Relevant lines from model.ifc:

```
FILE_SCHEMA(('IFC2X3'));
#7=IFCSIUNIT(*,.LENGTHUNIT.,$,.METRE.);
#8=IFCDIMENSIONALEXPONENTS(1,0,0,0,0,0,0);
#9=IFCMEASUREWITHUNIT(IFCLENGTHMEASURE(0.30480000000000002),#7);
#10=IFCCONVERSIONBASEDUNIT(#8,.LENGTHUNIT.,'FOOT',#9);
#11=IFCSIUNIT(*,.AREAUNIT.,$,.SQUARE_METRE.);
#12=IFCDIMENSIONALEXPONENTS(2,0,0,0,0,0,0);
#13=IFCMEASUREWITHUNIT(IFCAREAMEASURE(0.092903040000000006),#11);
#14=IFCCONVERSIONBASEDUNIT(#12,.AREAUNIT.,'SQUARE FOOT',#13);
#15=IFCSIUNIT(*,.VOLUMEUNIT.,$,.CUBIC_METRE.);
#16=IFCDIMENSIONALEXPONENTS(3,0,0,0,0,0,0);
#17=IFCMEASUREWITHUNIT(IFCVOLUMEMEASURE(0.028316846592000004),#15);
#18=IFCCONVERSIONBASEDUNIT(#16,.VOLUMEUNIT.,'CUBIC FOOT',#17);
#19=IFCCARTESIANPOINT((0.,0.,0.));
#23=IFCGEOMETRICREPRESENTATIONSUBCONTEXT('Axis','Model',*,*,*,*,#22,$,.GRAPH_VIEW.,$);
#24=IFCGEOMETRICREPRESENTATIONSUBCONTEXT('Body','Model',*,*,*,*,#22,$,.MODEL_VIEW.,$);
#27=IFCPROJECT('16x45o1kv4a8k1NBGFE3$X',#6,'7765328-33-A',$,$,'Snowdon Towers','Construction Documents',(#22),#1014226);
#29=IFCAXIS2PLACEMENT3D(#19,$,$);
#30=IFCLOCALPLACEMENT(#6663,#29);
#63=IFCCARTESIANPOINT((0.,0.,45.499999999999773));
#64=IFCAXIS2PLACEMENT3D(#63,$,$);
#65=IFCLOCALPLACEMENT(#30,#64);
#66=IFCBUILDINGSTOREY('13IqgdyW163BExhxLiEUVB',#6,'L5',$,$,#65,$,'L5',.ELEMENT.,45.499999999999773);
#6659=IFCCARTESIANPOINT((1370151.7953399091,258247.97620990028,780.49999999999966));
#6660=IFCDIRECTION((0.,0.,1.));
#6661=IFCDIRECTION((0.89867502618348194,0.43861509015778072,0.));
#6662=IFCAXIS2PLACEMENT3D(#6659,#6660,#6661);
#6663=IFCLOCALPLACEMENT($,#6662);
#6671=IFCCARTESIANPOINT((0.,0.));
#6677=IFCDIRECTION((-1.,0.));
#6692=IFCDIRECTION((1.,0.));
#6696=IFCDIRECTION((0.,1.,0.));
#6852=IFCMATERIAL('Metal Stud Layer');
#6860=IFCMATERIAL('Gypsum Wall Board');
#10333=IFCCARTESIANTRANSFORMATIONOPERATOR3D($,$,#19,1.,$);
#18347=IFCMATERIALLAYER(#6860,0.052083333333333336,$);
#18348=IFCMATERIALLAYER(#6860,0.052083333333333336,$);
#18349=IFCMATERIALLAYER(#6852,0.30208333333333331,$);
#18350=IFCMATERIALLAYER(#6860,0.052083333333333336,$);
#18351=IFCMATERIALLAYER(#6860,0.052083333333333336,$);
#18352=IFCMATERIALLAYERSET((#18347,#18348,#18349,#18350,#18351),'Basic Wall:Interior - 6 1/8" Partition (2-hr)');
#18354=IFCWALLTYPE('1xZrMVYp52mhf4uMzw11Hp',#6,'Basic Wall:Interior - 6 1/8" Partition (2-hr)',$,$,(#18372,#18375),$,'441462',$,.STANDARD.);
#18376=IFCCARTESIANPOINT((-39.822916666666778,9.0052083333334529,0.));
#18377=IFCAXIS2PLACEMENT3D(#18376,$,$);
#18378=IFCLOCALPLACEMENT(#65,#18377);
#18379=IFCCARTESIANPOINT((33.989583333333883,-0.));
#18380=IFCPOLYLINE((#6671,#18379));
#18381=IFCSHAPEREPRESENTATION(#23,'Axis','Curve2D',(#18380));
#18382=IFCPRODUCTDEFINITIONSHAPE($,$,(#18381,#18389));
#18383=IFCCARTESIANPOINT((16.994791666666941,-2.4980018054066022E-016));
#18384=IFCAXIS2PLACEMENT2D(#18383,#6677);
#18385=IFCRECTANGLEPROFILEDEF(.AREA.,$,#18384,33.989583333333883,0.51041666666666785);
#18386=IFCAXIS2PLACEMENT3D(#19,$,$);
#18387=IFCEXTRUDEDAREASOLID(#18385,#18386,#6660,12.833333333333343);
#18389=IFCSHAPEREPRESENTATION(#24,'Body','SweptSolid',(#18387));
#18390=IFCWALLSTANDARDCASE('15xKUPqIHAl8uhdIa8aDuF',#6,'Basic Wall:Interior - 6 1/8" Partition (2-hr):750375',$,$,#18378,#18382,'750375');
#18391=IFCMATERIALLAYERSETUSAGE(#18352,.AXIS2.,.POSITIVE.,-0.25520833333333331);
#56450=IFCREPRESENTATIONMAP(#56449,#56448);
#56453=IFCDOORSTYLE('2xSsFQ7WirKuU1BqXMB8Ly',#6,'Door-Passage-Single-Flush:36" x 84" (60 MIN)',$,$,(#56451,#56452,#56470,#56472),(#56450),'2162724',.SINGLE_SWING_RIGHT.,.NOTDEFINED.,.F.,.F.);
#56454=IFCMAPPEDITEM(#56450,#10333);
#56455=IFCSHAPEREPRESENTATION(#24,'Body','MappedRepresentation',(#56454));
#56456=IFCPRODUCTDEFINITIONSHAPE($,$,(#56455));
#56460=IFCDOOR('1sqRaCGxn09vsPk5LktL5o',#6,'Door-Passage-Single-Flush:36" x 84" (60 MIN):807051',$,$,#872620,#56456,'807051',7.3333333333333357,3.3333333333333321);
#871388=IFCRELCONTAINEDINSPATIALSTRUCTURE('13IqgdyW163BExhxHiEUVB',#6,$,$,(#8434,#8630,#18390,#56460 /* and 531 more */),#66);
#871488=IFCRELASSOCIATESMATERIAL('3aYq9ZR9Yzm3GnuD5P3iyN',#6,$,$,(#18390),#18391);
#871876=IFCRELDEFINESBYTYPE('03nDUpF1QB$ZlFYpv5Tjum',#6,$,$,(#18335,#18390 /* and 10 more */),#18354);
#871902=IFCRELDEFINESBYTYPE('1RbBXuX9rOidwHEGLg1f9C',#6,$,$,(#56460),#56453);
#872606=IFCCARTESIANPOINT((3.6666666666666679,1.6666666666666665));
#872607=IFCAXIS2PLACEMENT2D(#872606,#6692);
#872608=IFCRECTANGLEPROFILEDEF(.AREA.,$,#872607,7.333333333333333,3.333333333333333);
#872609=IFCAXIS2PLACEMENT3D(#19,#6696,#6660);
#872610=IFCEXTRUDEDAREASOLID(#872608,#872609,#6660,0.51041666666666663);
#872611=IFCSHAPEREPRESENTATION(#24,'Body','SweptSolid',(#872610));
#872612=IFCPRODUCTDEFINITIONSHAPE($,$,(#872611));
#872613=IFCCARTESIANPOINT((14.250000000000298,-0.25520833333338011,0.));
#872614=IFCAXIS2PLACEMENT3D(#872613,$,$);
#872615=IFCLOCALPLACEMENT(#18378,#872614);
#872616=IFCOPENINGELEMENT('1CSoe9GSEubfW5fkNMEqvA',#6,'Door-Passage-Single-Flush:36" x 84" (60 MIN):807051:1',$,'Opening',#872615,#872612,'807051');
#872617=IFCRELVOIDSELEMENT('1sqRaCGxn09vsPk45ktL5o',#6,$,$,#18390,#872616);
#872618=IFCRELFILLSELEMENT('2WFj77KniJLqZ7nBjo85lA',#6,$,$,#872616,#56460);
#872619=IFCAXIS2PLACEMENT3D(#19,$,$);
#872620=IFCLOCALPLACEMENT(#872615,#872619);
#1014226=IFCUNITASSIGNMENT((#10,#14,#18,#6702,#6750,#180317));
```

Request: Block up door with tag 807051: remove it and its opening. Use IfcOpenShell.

```python
import ifcopenshell
import ifcopenshell.api.feature
import ifcopenshell.api.root
import ifcopenshell.geom
import ifcopenshell.util.shape

model = ifcopenshell.open("model.ifc")
settings = ifcopenshell.geom.settings()


def volume(element):
    """Net volume in cubic metres, openings subtracted."""
    shape = ifcopenshell.geom.create_shape(settings, element)
    return ifcopenshell.util.shape.get_volume(shape.geometry)


door = model.by_guid("1sqRaCGxn09vsPk5LktL5o")
opening = door.FillsVoids[0].RelatingOpeningElement
wall = opening.VoidsElements[0].RelatingBuildingElement
before = volume(wall)

ifcopenshell.api.root.remove_product(model, product=door)
ifcopenshell.api.feature.remove_feature(model, feature=opening)

after = volume(wall)

print(f"wall volume {before:.3f} -> {after:.3f} m3")

model.write("model_updated.ifc")
```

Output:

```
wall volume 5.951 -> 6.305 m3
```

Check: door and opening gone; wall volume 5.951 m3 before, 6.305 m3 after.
